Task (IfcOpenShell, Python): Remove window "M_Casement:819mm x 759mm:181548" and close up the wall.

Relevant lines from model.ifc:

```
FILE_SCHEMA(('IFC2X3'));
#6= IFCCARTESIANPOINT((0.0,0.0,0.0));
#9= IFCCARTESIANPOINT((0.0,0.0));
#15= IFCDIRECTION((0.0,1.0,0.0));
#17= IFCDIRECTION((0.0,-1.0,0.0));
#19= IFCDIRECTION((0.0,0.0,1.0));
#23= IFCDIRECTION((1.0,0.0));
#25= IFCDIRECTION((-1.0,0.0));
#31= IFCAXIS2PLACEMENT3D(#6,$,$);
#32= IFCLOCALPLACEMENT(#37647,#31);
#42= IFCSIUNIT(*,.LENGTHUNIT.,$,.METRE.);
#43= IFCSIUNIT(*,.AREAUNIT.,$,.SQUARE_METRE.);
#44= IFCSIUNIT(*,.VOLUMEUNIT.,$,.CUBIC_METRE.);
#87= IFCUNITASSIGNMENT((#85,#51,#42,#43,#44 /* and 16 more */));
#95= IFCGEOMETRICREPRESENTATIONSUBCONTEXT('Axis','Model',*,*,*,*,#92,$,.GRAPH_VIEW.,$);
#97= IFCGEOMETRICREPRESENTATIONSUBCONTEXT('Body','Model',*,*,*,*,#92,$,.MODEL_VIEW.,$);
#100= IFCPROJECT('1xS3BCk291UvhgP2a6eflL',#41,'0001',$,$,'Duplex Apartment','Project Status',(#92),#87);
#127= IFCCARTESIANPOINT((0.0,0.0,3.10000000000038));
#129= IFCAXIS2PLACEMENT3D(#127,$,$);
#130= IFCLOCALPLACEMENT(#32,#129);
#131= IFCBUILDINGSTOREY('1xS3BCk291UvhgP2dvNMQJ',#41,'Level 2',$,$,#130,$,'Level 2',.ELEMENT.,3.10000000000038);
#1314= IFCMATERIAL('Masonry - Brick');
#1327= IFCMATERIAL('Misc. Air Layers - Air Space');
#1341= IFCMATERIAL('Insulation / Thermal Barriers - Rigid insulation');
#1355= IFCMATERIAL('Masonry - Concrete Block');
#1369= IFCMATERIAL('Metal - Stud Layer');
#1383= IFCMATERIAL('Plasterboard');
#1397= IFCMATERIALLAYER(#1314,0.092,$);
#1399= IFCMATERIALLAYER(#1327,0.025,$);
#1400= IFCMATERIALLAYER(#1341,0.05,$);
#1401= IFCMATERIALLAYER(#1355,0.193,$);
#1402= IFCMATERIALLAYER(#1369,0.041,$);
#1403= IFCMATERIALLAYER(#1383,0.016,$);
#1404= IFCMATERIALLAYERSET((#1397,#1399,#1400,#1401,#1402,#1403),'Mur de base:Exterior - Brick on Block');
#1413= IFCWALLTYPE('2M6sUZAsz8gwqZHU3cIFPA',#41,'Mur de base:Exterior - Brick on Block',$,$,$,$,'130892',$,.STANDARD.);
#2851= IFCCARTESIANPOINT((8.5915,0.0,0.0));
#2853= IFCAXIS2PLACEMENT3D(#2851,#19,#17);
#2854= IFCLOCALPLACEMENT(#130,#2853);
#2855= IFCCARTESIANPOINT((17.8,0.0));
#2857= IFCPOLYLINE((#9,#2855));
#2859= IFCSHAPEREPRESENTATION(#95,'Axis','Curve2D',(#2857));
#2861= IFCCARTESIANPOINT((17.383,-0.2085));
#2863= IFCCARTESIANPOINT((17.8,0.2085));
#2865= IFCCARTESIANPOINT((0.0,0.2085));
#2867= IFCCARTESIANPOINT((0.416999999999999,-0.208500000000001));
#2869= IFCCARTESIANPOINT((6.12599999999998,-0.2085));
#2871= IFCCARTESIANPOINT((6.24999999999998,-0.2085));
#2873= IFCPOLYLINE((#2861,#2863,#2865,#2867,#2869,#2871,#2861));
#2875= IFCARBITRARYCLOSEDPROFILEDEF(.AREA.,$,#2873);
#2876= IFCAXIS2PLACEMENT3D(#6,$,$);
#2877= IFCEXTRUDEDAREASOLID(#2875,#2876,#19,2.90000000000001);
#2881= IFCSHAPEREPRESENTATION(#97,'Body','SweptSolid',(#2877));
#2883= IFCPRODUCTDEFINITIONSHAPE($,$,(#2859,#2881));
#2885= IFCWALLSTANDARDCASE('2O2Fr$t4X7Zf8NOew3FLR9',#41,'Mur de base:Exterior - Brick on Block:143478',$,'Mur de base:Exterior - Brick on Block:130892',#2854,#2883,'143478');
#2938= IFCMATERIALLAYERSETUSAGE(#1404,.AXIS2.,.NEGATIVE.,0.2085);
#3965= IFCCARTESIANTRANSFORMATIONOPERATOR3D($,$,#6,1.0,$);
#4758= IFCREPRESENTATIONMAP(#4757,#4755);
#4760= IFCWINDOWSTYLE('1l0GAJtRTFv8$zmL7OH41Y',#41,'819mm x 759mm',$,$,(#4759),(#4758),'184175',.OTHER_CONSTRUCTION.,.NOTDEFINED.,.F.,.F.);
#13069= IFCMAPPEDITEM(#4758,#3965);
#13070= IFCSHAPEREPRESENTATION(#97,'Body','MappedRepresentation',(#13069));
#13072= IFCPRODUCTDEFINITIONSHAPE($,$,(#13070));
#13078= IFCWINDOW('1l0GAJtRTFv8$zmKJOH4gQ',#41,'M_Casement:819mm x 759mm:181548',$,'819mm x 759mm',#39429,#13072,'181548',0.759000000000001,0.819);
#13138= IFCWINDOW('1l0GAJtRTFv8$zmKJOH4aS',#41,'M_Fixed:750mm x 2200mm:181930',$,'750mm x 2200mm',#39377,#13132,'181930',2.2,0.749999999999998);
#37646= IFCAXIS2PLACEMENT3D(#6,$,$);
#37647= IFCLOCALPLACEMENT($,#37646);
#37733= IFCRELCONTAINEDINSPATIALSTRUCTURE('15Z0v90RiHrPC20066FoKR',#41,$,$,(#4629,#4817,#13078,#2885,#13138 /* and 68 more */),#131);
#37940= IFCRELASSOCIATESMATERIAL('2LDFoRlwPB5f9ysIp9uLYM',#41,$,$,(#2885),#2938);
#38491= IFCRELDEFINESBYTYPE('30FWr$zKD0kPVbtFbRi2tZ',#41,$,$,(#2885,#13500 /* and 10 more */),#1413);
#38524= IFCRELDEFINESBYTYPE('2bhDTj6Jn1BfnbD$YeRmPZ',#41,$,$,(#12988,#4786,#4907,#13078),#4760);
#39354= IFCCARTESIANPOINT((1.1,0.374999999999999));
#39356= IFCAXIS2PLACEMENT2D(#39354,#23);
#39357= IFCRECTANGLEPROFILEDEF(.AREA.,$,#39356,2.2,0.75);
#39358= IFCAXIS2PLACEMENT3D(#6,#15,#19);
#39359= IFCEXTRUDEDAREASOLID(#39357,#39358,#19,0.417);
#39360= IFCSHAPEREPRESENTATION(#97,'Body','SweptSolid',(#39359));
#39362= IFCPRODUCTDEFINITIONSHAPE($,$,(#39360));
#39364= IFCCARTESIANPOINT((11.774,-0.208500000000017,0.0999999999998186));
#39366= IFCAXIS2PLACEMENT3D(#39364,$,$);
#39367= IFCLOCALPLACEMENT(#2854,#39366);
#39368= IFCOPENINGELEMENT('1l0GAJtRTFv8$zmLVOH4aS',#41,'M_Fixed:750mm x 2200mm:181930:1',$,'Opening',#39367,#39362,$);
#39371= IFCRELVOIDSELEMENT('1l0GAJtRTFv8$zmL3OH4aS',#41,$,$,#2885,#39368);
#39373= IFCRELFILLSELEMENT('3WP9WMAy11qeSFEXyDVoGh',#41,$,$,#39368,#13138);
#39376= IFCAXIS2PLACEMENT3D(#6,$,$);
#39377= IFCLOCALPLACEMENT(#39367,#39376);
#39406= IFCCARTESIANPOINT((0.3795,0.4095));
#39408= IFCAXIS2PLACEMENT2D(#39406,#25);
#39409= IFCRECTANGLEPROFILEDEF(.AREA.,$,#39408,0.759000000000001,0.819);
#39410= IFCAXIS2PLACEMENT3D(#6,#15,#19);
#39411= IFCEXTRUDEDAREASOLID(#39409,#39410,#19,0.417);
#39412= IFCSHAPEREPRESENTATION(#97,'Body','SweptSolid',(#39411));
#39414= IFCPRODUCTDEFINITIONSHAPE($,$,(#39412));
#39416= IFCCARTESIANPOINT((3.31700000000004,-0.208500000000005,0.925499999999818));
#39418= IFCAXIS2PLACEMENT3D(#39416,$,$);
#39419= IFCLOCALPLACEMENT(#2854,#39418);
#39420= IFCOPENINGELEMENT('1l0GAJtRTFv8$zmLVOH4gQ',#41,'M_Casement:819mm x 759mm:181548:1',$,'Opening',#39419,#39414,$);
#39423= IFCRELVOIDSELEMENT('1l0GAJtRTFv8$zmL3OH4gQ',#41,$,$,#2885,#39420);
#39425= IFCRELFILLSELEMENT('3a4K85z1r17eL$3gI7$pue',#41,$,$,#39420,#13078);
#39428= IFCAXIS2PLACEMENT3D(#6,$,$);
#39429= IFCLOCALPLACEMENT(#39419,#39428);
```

```python
import ifcopenshell
import ifcopenshell.api.feature
import ifcopenshell.api.root
import ifcopenshell.geom
import ifcopenshell.util.shape

model = ifcopenshell.open("model.ifc")
settings = ifcopenshell.geom.settings()


def volume(element):
    """Net volume in cubic metres, openings subtracted."""
    shape = ifcopenshell.geom.create_shape(settings, element)
    return ifcopenshell.util.shape.get_volume(shape.geometry)


window = model.by_guid("1l0GAJtRTFv8$zmKJOH4gQ")
opening = window.FillsVoids[0].RelatingOpeningElement
wall = opening.VoidsElements[0].RelatingBuildingElement
before = volume(wall)

ifcopenshell.api.root.remove_product(model, product=window)
ifcopenshell.api.feature.remove_feature(model, feature=opening)

after = volume(wall)

print(f"wall volume {before:.3f} -> {after:.3f} m3")

model.write("model_updated.ifc")
```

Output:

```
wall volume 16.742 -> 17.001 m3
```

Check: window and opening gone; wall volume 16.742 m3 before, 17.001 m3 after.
